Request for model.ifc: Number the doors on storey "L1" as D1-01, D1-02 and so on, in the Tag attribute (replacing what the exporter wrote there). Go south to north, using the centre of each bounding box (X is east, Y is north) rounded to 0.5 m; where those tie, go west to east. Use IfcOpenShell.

First a look at what the model holds.

```python
import ifcopenshell
import ifcopenshell.util.element
import ifcopenshell.util.placement

model = ifcopenshell.open("model.ifc")
print(model.schema)
storey = next(s for s in model.by_type("IfcBuildingStorey") if s.Name == "L1")
doors = [e for e in ifcopenshell.util.element.get_decomposition(storey) if e.is_a("IfcDoor")]
for e in sorted(doors, key=lambda e: e.id()):
    origin = ifcopenshell.util.placement.get_local_placement(e.ObjectPlacement)[:3, 3]
    print(e.id(), e.Tag, e.Name, origin.round(2) + 0.0, sep=" | ")
```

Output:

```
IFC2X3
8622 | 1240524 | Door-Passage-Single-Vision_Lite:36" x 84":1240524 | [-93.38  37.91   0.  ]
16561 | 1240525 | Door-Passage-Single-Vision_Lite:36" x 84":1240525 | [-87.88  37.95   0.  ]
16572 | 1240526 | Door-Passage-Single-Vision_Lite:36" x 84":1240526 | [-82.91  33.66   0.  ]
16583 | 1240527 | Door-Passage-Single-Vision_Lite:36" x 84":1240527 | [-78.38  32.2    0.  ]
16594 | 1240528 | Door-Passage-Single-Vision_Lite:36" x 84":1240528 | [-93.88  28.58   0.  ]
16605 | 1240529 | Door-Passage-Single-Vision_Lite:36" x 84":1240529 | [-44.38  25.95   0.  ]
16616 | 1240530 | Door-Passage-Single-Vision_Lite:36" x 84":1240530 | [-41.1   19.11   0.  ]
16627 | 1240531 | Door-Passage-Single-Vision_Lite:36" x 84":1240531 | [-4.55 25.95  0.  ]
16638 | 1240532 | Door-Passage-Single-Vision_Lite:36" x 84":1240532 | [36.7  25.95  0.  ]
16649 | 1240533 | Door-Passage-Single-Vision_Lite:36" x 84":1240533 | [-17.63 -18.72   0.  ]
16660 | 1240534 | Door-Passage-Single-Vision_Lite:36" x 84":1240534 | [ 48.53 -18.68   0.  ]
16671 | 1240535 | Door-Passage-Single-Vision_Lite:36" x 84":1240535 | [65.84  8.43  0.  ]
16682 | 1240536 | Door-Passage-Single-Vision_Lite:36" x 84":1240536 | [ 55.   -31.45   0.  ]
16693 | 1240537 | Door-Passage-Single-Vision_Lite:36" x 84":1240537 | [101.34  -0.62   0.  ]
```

```python
import ifcopenshell
import ifcopenshell.geom
import ifcopenshell.util.element
import ifcopenshell.util.shape

model = ifcopenshell.open("model.ifc")
settings = ifcopenshell.geom.settings()
settings.set("use-world-coords", True)


def centre(element):
    shape = ifcopenshell.geom.create_shape(settings, element)
    return ifcopenshell.util.shape.get_bbox_centroid(shape.geometry)


storey = next(s for s in model.by_type("IfcBuildingStorey") if s.Name == "L1")
doors = [e for e in ifcopenshell.util.element.get_decomposition(storey) if e.is_a("IfcDoor")]

# Insertion points can sit at a corner or the storey origin, so sort by the geometry (in metres).
centres = {e: centre(e) for e in doors}
doors.sort(key=lambda e: (round(centres[e][1] / 0.5), centres[e][0]))

for i, e in enumerate(doors, start=1):
    number = f"D1-{i:02d}"
    e.Tag = number
    print(e.id(), number)

model.write("model_edited.ifc")
```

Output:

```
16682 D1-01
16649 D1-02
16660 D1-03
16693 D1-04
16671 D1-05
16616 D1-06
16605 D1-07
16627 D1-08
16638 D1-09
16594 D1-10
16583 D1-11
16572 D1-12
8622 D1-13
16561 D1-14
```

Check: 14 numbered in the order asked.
